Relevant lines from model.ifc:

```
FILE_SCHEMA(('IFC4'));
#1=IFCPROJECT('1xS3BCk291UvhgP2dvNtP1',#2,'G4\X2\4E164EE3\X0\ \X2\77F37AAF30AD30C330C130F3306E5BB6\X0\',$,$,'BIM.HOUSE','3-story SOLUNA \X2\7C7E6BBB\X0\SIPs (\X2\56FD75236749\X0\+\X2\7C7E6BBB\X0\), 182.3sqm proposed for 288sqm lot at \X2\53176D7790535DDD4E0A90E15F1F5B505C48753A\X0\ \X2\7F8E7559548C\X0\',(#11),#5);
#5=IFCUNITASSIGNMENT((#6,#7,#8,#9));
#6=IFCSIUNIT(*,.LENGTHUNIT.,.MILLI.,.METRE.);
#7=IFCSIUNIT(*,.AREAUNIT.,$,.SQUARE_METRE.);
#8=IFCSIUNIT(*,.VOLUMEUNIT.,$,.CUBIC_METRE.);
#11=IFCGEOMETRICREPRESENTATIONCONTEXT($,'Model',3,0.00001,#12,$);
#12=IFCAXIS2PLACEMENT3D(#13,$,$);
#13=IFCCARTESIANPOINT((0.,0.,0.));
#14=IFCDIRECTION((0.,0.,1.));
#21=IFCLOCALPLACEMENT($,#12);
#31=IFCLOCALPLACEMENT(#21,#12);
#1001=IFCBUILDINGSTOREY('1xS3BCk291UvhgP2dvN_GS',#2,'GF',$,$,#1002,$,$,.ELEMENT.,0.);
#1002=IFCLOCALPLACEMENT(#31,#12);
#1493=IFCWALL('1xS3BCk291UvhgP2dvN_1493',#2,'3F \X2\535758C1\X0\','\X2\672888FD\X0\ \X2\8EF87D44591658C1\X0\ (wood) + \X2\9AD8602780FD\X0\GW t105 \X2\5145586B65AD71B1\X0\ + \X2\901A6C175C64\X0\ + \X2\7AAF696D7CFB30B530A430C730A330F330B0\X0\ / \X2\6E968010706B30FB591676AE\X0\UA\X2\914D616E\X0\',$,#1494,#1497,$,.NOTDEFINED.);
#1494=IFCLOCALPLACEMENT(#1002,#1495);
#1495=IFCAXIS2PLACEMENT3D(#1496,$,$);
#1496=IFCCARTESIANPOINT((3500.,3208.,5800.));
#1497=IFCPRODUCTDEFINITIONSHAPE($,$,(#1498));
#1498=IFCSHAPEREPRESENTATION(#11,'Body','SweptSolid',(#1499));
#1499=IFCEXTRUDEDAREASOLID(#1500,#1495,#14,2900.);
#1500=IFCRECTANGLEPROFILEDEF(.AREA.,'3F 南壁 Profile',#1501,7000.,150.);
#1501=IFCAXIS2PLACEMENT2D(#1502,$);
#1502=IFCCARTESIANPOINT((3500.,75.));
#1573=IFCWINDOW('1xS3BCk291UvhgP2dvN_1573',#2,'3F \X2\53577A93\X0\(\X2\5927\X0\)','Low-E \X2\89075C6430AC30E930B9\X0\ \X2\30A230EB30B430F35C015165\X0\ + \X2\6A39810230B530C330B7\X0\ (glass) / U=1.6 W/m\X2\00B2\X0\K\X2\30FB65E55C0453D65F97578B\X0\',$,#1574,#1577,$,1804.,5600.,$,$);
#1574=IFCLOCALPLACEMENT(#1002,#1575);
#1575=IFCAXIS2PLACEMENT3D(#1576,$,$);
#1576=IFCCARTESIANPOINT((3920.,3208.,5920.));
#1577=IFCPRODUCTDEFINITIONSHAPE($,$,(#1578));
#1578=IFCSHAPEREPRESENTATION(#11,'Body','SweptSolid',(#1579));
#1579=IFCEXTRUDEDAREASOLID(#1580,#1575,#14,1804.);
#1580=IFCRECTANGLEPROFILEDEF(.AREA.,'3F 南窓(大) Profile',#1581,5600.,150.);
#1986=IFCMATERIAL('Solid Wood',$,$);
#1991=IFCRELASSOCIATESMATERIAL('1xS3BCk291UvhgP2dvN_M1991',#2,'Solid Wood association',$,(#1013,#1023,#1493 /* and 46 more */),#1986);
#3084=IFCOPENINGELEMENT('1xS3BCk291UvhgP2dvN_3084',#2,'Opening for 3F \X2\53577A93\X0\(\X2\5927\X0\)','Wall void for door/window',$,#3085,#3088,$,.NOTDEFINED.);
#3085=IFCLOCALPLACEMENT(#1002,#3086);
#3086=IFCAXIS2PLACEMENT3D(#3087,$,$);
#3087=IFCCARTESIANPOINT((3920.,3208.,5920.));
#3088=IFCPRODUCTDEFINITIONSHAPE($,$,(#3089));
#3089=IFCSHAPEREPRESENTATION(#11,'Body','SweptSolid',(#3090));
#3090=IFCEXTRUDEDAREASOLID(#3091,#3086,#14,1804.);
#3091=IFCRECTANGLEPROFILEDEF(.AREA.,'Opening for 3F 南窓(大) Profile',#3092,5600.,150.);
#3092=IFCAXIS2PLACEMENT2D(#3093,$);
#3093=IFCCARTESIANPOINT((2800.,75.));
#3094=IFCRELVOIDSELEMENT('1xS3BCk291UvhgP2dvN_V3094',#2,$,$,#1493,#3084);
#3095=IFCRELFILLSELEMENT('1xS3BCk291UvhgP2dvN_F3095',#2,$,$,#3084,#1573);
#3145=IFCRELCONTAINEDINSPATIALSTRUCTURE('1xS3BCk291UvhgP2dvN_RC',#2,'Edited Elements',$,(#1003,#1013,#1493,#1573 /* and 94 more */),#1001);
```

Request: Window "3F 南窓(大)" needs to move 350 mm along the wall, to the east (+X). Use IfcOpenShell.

```python
import ifcopenshell
import ifcopenshell.api.geometry
import ifcopenshell.util.placement
import ifcopenshell.util.unit

model = ifcopenshell.open("model.ifc")
unit_scale = ifcopenshell.util.unit.calculate_unit_scale(model)

window = model.by_guid("1xS3BCk291UvhgP2dvN_1573")
opening = window.FillsVoids[0].RelatingOpeningElement
wall = opening.VoidsElements[0].RelatingBuildingElement

wall_matrix = ifcopenshell.util.placement.get_local_placement(wall.ObjectPlacement)
shift = wall_matrix[:3, 0] * 0.35 / unit_scale
before = ifcopenshell.util.placement.get_local_placement(window.ObjectPlacement)[:3, 3].copy()

# The window is not placed relative to its opening, so move both.
for product in (opening, window):
    matrix = ifcopenshell.util.placement.get_local_placement(product.ObjectPlacement)
    matrix[:3, 3] += shift
    ifcopenshell.api.geometry.edit_object_placement(model, product=product, matrix=matrix, is_si=False)

after = ifcopenshell.util.placement.get_local_placement(window.ObjectPlacement)[:3, 3]
print("window moved by", (after - before).round(3) + 0.0)

model.write("model-out.ifc")
```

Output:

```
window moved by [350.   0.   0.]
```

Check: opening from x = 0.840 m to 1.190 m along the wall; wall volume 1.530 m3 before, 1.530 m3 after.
